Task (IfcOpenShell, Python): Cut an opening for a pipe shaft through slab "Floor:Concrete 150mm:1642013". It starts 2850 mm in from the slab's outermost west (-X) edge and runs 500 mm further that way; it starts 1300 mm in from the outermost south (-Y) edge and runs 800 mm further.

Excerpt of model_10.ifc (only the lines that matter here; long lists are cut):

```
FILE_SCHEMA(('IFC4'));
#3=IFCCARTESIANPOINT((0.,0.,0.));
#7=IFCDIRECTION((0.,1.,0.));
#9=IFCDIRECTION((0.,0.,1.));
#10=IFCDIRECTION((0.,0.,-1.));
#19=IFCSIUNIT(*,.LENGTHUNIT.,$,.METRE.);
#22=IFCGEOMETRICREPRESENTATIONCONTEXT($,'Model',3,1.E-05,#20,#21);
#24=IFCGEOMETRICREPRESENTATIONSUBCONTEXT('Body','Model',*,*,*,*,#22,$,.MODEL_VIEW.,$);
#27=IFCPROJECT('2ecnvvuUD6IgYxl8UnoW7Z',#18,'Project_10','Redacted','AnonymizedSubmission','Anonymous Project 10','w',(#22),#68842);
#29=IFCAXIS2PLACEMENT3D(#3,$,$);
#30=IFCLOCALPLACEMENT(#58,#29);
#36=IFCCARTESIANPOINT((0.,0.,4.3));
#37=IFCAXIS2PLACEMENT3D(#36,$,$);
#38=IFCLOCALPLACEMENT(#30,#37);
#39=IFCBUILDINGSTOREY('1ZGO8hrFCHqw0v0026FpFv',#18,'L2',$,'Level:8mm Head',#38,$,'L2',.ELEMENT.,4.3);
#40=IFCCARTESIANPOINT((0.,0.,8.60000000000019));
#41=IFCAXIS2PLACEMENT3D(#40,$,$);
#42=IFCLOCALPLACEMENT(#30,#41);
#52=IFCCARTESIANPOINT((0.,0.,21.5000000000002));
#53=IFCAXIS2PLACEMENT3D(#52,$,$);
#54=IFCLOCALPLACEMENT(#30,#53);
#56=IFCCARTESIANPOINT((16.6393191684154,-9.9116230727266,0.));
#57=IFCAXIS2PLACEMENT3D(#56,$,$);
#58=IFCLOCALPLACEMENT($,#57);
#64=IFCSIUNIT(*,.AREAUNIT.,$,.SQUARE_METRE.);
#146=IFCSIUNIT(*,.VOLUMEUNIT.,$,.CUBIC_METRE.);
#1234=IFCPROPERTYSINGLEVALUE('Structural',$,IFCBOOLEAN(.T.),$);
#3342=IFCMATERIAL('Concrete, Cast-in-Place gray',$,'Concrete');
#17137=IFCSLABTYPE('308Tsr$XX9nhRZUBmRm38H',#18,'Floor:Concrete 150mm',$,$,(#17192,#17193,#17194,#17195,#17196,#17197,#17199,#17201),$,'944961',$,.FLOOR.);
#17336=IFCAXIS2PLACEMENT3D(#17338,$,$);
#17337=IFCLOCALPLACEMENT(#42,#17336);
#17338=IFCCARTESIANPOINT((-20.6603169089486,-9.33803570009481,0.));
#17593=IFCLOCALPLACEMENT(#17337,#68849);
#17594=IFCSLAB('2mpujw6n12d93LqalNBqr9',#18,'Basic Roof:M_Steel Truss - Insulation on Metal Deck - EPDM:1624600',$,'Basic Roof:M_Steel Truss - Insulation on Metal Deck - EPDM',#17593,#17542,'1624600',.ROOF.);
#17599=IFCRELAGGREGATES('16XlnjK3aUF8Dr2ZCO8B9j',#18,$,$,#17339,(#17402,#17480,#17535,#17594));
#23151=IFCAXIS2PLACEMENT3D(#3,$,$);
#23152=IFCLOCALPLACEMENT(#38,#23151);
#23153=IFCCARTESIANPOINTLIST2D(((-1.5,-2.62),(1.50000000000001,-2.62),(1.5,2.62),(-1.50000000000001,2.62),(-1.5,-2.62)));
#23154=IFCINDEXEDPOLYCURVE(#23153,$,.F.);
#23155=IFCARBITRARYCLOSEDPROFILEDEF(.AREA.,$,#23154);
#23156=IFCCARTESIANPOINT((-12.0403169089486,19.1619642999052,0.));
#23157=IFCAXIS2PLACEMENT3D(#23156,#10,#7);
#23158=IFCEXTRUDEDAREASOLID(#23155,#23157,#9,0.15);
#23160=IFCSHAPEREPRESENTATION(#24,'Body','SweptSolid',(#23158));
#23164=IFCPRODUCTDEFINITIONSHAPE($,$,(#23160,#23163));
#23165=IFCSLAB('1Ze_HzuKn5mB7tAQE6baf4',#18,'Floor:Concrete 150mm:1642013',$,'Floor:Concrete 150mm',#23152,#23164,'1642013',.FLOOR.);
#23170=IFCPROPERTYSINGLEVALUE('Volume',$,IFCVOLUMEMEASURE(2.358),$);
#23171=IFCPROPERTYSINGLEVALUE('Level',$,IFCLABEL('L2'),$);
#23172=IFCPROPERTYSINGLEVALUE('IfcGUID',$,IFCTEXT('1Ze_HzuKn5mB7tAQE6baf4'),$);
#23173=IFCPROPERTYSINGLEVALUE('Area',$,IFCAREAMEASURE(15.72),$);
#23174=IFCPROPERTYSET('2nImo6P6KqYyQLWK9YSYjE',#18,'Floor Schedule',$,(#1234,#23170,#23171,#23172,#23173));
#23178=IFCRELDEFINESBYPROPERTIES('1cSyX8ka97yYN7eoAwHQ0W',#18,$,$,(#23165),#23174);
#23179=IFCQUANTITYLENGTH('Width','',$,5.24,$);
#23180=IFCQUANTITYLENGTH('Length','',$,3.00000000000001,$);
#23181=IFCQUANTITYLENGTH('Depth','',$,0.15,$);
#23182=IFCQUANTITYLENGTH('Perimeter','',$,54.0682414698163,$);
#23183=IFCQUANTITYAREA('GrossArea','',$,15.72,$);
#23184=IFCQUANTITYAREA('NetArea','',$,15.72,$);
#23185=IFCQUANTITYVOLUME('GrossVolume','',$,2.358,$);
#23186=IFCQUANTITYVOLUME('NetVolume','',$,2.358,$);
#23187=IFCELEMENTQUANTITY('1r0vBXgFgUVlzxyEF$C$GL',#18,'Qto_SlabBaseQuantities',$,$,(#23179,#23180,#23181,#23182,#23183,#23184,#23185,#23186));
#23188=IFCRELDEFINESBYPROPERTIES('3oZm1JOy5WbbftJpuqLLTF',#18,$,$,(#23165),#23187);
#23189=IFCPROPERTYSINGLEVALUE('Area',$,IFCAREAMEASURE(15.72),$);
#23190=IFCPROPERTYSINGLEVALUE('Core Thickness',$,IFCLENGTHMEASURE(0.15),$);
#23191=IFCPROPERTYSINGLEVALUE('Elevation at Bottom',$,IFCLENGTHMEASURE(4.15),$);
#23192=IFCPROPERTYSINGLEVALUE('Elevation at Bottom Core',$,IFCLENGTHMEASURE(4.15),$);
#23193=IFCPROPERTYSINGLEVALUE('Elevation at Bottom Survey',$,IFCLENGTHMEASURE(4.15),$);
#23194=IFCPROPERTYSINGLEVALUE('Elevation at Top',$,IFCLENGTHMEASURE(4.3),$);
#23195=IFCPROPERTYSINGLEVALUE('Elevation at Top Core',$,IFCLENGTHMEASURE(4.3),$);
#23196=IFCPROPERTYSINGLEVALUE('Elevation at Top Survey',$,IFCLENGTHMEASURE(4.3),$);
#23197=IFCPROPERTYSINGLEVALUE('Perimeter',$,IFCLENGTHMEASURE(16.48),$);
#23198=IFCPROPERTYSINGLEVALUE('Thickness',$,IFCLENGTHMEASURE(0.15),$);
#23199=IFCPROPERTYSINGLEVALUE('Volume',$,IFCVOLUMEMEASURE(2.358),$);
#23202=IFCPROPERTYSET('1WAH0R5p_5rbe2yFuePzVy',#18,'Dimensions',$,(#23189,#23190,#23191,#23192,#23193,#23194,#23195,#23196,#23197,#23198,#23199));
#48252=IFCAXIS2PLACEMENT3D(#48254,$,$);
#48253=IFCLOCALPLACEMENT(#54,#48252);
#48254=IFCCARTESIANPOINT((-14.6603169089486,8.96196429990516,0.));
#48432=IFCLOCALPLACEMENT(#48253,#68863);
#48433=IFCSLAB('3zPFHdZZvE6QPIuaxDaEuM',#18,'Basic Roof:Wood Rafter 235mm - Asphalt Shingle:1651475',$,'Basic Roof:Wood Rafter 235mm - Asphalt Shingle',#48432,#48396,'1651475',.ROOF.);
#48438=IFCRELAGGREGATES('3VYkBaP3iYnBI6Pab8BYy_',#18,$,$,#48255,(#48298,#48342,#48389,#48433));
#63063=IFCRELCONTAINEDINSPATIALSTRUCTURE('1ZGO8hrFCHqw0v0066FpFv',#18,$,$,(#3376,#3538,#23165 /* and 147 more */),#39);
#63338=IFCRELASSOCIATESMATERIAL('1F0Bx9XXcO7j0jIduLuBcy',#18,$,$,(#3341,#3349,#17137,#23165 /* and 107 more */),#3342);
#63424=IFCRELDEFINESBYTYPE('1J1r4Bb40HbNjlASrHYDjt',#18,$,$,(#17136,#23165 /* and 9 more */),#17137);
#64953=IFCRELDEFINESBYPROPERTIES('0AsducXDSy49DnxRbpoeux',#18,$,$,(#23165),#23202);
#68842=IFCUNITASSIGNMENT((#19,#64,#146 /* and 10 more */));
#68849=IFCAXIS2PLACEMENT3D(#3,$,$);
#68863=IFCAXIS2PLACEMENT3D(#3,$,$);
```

```python
import numpy as np
import ifcopenshell
import ifcopenshell.api.feature
import ifcopenshell.api.geometry
import ifcopenshell.api.pset
import ifcopenshell.api.root
import ifcopenshell.geom
import ifcopenshell.util.element
import ifcopenshell.util.placement
import ifcopenshell.util.representation
import ifcopenshell.util.shape
import ifcopenshell.util.unit

model = ifcopenshell.open("model_10.ifc")
unit_scale = ifcopenshell.util.unit.calculate_unit_scale(model)
area_scale = ifcopenshell.util.unit.calculate_unit_scale(model, "AREAUNIT")
volume_scale = ifcopenshell.util.unit.calculate_unit_scale(model, "VOLUMEUNIT")
settings = ifcopenshell.geom.settings()


def volume(element):
    """Net volume in cubic metres, openings subtracted."""
    shape = ifcopenshell.geom.create_shape(settings, element)
    return ifcopenshell.util.shape.get_volume(shape.geometry)


slab = model.by_guid("1Ze_HzuKn5mB7tAQE6baf4")
before = volume(slab)

# Extent in the slab's own axes, in metres. The edges named are its -X and -Y sides.
slab_shape = ifcopenshell.geom.create_shape(settings, slab)
vertices = ifcopenshell.util.shape.get_vertices(slab_shape.geometry)
x_min, y_min, bottom = vertices.min(axis=0)
top = vertices[:, 2].max()

opening = ifcopenshell.api.root.create_entity(model, ifc_class="IfcOpeningElement", name="Pipe shaft opening", predefined_type="OPENING")
context = ifcopenshell.util.representation.get_context(model, "Model", "Body", "MODEL_VIEW")
width, depth = 0.5, 0.8
outline = [(0.0, 0.0), (width, 0.0), (width, depth), (0.0, depth), (0.0, 0.0)]
# Overshoot both faces by 50 mm so the cut is clean.
shape = ifcopenshell.api.geometry.add_slab_representation(
    model, context=context, depth=top - bottom + 0.1, polyline=outline
)
ifcopenshell.api.geometry.assign_representation(model, product=opening, representation=shape)

matrix = ifcopenshell.util.placement.get_local_placement(slab.ObjectPlacement)
matrix[:, 3] = matrix @ np.append(np.array([x_min + 2.85, y_min + 1.3, bottom - 0.05]) / unit_scale, 1.0)
ifcopenshell.api.geometry.edit_object_placement(model, product=opening, matrix=matrix, is_si=False)
ifcopenshell.api.feature.add_feature(model, feature=opening, element=slab)

after = volume(slab)

# Update the slab's stored quantities.
pset = model.by_id(ifcopenshell.util.element.get_pset(slab, "Floor Schedule", should_inherit=False)["id"])
ifcopenshell.api.pset.edit_pset(model, pset=pset, properties={
    "Volume": model.create_entity("IfcVolumeMeasure", after / volume_scale),
    "Area": model.create_entity("IfcAreaMeasure", after / (top - bottom) / area_scale),
})
qto = model.by_id(ifcopenshell.util.element.get_pset(slab, "Qto_SlabBaseQuantities", should_inherit=False)["id"])
ifcopenshell.api.pset.edit_qto(model, qto=qto, properties={
    "NetArea": after / (top - bottom) / area_scale,
    "NetVolume": after / volume_scale,
})
pset = model.by_id(ifcopenshell.util.element.get_pset(slab, "Dimensions", should_inherit=False)["id"])
ifcopenshell.api.pset.edit_pset(model, pset=pset, properties={
    "Area": model.create_entity("IfcAreaMeasure", after / (top - bottom) / area_scale),
    "Volume": model.create_entity("IfcVolumeMeasure", after / volume_scale),
})

print(f"slab volume {before:.3f} -> {after:.3f} m3")

model.write("model_10-out.ifc")
```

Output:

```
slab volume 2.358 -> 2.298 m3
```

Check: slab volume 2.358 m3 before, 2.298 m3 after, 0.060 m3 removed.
